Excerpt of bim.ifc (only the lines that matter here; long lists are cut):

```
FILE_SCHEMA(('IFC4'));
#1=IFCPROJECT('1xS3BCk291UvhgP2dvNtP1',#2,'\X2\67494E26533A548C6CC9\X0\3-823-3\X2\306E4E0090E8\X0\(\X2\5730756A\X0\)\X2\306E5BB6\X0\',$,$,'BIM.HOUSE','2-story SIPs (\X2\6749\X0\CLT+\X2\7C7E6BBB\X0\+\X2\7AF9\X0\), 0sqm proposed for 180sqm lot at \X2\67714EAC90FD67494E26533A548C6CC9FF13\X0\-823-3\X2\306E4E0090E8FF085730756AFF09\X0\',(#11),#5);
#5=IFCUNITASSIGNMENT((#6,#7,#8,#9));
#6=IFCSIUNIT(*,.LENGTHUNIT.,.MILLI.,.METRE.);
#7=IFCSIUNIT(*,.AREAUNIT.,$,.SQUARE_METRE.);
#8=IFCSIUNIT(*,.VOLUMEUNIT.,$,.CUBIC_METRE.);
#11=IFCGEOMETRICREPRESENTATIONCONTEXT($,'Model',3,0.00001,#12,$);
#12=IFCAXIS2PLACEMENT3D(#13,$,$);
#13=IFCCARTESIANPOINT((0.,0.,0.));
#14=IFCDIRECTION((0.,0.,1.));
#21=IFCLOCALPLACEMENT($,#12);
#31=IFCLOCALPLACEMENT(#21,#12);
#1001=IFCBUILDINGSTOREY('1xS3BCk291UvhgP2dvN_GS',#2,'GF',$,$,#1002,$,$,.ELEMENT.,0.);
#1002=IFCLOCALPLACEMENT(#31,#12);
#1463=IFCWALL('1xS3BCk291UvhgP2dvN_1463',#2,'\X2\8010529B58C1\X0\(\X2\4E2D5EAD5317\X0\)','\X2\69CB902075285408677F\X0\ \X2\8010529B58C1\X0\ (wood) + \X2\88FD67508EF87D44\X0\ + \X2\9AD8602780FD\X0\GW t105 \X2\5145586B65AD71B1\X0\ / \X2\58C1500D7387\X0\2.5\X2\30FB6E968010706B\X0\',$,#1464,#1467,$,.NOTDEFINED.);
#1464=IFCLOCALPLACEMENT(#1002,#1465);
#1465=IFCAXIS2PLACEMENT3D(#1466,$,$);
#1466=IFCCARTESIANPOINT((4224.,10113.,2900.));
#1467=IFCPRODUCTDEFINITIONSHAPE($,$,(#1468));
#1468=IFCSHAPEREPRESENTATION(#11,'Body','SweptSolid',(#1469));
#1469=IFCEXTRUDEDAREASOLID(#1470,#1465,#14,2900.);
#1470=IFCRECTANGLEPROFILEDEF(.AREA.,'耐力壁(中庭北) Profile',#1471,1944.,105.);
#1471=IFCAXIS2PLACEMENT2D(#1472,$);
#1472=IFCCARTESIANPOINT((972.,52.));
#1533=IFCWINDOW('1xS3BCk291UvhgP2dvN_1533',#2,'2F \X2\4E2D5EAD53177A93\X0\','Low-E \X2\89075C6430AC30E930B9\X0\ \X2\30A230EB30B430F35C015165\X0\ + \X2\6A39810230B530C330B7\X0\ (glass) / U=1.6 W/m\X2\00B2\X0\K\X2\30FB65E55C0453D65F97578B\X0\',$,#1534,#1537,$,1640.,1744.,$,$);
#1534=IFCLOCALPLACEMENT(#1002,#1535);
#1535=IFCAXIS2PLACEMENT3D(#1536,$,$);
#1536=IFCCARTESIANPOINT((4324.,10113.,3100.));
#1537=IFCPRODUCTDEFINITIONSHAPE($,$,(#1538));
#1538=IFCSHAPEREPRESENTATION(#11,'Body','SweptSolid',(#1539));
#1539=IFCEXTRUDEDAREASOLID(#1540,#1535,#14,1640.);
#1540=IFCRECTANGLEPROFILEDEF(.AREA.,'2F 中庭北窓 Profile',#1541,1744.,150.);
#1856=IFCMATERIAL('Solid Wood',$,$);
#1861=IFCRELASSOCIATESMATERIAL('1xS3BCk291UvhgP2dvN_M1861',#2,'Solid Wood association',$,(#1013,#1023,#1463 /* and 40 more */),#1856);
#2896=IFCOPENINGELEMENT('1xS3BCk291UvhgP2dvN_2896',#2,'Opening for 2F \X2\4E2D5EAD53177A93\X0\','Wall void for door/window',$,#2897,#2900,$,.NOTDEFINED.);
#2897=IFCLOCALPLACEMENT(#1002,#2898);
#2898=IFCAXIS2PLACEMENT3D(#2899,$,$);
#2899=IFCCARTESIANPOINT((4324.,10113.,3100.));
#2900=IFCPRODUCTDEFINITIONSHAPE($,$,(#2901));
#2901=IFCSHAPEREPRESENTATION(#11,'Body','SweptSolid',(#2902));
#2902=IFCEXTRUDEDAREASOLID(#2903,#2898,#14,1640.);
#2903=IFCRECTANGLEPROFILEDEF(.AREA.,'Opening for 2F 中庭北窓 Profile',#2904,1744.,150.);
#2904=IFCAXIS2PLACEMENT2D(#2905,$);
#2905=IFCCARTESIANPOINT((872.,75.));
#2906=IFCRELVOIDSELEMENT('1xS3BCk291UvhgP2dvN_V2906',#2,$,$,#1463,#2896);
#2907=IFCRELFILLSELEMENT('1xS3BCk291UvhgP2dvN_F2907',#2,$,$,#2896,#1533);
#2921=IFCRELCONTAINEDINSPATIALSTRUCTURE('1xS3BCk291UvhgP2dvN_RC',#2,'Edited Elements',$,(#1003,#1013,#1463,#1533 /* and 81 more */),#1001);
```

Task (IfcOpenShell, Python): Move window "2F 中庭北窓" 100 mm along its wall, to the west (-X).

```python
import ifcopenshell
import ifcopenshell.api.geometry
import ifcopenshell.util.placement
import ifcopenshell.util.unit

model = ifcopenshell.open("bim.ifc")
unit_scale = ifcopenshell.util.unit.calculate_unit_scale(model)

window = model.by_id(1533)
opening = window.FillsVoids[0].RelatingOpeningElement
wall = opening.VoidsElements[0].RelatingBuildingElement

wall_matrix = ifcopenshell.util.placement.get_local_placement(wall.ObjectPlacement)
shift = wall_matrix[:3, 0] * -0.1 / unit_scale
before = ifcopenshell.util.placement.get_local_placement(window.ObjectPlacement)[:3, 3].copy()

# The window is not placed relative to its opening, so move both.
for product in (opening, window):
    matrix = ifcopenshell.util.placement.get_local_placement(product.ObjectPlacement)
    matrix[:3, 3] += shift
    ifcopenshell.api.geometry.edit_object_placement(model, product=product, matrix=matrix, is_si=False)

after = ifcopenshell.util.placement.get_local_placement(window.ObjectPlacement)[:3, 3]
print("window moved by", (after - before).round(3) + 0.0)

model.write("bim_v2.ifc")
```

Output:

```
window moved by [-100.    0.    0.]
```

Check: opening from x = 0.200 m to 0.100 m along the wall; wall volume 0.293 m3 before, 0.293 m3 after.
